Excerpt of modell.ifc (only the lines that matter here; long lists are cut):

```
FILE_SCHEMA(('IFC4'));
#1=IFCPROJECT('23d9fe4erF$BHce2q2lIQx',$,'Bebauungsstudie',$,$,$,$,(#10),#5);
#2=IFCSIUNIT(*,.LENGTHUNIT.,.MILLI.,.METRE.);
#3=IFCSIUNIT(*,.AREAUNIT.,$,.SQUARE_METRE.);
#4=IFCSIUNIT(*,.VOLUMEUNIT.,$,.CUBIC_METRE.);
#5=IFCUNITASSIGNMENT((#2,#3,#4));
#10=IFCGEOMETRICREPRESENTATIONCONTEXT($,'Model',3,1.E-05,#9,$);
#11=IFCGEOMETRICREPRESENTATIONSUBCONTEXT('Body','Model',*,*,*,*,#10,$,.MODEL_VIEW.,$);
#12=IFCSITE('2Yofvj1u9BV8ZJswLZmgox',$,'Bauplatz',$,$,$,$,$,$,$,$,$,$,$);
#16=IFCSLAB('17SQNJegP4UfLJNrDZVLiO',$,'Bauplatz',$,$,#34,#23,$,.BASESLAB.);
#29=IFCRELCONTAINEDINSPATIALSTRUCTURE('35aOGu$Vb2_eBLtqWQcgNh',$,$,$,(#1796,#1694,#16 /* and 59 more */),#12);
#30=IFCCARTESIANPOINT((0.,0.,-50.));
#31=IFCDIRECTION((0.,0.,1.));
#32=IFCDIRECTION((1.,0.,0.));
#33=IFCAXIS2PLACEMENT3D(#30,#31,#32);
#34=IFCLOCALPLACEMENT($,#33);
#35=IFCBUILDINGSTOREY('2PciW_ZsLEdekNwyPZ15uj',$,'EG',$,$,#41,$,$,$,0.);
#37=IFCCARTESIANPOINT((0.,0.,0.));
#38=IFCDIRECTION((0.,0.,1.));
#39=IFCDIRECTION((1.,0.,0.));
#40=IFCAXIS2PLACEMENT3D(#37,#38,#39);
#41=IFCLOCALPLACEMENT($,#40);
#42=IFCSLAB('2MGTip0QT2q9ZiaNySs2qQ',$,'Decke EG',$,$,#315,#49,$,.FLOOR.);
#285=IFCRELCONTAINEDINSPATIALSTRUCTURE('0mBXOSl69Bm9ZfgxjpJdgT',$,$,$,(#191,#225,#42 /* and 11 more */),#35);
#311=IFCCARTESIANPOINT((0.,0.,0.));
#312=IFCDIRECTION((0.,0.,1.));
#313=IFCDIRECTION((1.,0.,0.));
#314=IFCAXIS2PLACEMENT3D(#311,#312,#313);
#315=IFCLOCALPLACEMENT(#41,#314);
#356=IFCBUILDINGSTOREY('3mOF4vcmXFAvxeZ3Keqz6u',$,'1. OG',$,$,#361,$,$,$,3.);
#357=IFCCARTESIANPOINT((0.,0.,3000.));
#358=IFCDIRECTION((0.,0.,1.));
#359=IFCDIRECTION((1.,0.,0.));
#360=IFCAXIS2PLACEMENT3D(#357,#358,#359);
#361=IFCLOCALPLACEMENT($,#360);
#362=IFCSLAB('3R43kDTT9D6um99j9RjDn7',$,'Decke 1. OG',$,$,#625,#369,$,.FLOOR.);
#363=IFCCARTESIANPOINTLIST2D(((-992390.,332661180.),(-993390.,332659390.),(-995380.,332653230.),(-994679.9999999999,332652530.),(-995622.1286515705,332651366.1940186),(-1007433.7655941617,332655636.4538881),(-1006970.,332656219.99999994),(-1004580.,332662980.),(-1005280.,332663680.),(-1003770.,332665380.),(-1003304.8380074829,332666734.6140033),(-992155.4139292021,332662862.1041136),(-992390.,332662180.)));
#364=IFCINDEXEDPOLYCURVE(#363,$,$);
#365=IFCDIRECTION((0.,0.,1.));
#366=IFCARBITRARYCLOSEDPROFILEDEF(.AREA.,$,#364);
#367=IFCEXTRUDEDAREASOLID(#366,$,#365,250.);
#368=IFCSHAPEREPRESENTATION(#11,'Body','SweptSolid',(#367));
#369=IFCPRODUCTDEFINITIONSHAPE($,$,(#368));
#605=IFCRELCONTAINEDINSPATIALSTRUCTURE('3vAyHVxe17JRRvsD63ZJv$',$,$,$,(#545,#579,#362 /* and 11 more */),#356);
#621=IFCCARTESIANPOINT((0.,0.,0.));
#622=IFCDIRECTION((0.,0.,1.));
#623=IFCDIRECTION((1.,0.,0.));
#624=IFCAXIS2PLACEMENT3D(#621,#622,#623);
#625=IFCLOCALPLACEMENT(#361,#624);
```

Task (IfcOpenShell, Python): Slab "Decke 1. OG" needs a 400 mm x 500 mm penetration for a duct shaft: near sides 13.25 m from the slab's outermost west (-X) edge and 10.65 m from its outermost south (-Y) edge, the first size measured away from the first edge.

```python
import numpy as np
import ifcopenshell
import ifcopenshell.api.feature
import ifcopenshell.api.geometry
import ifcopenshell.api.root
import ifcopenshell.geom
import ifcopenshell.util.placement
import ifcopenshell.util.representation
import ifcopenshell.util.shape
import ifcopenshell.util.unit

model = ifcopenshell.open("modell.ifc")
unit_scale = ifcopenshell.util.unit.calculate_unit_scale(model)
settings = ifcopenshell.geom.settings()


def volume(element):
    """Net volume in cubic metres, openings subtracted."""
    shape = ifcopenshell.geom.create_shape(settings, element)
    return ifcopenshell.util.shape.get_volume(shape.geometry)


slab = model.by_guid("3R43kDTT9D6um99j9RjDn7")
before = volume(slab)

# Extent in the slab's own axes, in metres. The edges named are its -X and -Y sides.
slab_shape = ifcopenshell.geom.create_shape(settings, slab)
vertices = ifcopenshell.util.shape.get_vertices(slab_shape.geometry)
x_min, y_min, bottom = vertices.min(axis=0)
top = vertices[:, 2].max()

opening = ifcopenshell.api.root.create_entity(model, ifc_class="IfcOpeningElement", name="Duct shaft opening", predefined_type="OPENING")
context = ifcopenshell.util.representation.get_context(model, "Model", "Body", "MODEL_VIEW")
width, depth = 0.4, 0.5
outline = [(0.0, 0.0), (width, 0.0), (width, depth), (0.0, depth), (0.0, 0.0)]
# Overshoot both faces by 50 mm so the cut is clean.
shape = ifcopenshell.api.geometry.add_slab_representation(
    model, context=context, depth=top - bottom + 0.1, polyline=outline
)
ifcopenshell.api.geometry.assign_representation(model, product=opening, representation=shape)

matrix = ifcopenshell.util.placement.get_local_placement(slab.ObjectPlacement)
matrix[:, 3] = matrix @ np.append(np.array([x_min + 13.25, y_min + 10.65, bottom - 0.05]) / unit_scale, 1.0)
ifcopenshell.api.geometry.edit_object_placement(model, product=opening, matrix=matrix, is_si=False)
ifcopenshell.api.feature.add_feature(model, feature=opening, element=slab)

after = volume(slab)

print(f"slab volume {before:.3f} -> {after:.3f} m3")

model.write("modell_updated.ifc")
```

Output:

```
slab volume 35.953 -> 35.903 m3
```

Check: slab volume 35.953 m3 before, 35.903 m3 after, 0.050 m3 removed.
